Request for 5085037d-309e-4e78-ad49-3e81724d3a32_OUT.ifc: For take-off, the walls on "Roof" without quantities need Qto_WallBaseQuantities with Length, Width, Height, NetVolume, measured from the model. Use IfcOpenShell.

First a look at what the model holds.

```python
import ifcopenshell
import ifcopenshell.util.element
import ifcopenshell.util.unit

model = ifcopenshell.open("5085037d-309e-4e78-ad49-3e81724d3a32_OUT.ifc")
print(model.schema)
for unit_type in ("LENGTHUNIT", "AREAUNIT", "VOLUMEUNIT"):
    print(unit_type, ifcopenshell.util.unit.calculate_unit_scale(model, unit_type))
storey = next(s for s in model.by_type("IfcBuildingStorey") if s.Name == "Roof")
walls = [e for e in ifcopenshell.util.element.get_decomposition(storey) if e.is_a("IfcWall")]
for e in sorted(walls, key=lambda e: e.id()):
    print(e.id(), e.is_a(), e.Name, list(ifcopenshell.util.element.get_psets(e, qtos_only=True)), sep=" | ")
```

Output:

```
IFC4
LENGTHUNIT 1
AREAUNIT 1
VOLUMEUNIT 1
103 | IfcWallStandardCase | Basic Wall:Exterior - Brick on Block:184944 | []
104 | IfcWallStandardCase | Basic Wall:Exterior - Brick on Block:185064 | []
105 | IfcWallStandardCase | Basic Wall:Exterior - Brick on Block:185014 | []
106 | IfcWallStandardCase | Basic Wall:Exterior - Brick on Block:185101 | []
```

```python
import ifcopenshell
import ifcopenshell.api.pset
import ifcopenshell.geom
import ifcopenshell.util.element
import ifcopenshell.util.shape
import ifcopenshell.util.unit

model = ifcopenshell.open("5085037d-309e-4e78-ad49-3e81724d3a32_OUT.ifc")
unit_scale = ifcopenshell.util.unit.calculate_unit_scale(model)
volume_scale = ifcopenshell.util.unit.calculate_unit_scale(model, "VOLUMEUNIT")
settings = ifcopenshell.geom.settings()

storey = next(s for s in model.by_type("IfcBuildingStorey") if s.Name == "Roof")
walls = [e for e in ifcopenshell.util.element.get_decomposition(storey) if e.is_a("IfcWall")]

for e in sorted(walls, key=lambda e: e.id()):
    if ifcopenshell.util.element.get_psets(e, qtos_only=True, should_inherit=False):
        continue
    # Geometry comes back in metres, in the element's own axes.
    shape = ifcopenshell.geom.create_shape(settings, e)
    values = {
        "Length": ifcopenshell.util.shape.get_x(shape.geometry) / unit_scale,
        "Width": ifcopenshell.util.shape.get_y(shape.geometry) / unit_scale,
        "Height": ifcopenshell.util.shape.get_z(shape.geometry) / unit_scale,
        "NetVolume": ifcopenshell.util.shape.get_volume(shape.geometry) / volume_scale,
    }
    qto = ifcopenshell.api.pset.add_qto(model, product=e, name="Qto_WallBaseQuantities")
    ifcopenshell.api.pset.edit_qto(model, qto=qto, properties=values)
    print(e.id(), {k: round(v, 3) for k, v in values.items()})

model.write("5085037d-309e-4e78-ad49-3e81724d3a32_OUT_updated.ifc")
```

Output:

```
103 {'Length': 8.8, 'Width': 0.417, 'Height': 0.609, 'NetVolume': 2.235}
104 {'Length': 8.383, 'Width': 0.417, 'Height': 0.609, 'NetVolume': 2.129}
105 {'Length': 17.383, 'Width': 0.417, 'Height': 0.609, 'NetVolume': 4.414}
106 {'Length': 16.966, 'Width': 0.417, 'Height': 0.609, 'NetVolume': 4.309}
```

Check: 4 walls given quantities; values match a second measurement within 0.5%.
